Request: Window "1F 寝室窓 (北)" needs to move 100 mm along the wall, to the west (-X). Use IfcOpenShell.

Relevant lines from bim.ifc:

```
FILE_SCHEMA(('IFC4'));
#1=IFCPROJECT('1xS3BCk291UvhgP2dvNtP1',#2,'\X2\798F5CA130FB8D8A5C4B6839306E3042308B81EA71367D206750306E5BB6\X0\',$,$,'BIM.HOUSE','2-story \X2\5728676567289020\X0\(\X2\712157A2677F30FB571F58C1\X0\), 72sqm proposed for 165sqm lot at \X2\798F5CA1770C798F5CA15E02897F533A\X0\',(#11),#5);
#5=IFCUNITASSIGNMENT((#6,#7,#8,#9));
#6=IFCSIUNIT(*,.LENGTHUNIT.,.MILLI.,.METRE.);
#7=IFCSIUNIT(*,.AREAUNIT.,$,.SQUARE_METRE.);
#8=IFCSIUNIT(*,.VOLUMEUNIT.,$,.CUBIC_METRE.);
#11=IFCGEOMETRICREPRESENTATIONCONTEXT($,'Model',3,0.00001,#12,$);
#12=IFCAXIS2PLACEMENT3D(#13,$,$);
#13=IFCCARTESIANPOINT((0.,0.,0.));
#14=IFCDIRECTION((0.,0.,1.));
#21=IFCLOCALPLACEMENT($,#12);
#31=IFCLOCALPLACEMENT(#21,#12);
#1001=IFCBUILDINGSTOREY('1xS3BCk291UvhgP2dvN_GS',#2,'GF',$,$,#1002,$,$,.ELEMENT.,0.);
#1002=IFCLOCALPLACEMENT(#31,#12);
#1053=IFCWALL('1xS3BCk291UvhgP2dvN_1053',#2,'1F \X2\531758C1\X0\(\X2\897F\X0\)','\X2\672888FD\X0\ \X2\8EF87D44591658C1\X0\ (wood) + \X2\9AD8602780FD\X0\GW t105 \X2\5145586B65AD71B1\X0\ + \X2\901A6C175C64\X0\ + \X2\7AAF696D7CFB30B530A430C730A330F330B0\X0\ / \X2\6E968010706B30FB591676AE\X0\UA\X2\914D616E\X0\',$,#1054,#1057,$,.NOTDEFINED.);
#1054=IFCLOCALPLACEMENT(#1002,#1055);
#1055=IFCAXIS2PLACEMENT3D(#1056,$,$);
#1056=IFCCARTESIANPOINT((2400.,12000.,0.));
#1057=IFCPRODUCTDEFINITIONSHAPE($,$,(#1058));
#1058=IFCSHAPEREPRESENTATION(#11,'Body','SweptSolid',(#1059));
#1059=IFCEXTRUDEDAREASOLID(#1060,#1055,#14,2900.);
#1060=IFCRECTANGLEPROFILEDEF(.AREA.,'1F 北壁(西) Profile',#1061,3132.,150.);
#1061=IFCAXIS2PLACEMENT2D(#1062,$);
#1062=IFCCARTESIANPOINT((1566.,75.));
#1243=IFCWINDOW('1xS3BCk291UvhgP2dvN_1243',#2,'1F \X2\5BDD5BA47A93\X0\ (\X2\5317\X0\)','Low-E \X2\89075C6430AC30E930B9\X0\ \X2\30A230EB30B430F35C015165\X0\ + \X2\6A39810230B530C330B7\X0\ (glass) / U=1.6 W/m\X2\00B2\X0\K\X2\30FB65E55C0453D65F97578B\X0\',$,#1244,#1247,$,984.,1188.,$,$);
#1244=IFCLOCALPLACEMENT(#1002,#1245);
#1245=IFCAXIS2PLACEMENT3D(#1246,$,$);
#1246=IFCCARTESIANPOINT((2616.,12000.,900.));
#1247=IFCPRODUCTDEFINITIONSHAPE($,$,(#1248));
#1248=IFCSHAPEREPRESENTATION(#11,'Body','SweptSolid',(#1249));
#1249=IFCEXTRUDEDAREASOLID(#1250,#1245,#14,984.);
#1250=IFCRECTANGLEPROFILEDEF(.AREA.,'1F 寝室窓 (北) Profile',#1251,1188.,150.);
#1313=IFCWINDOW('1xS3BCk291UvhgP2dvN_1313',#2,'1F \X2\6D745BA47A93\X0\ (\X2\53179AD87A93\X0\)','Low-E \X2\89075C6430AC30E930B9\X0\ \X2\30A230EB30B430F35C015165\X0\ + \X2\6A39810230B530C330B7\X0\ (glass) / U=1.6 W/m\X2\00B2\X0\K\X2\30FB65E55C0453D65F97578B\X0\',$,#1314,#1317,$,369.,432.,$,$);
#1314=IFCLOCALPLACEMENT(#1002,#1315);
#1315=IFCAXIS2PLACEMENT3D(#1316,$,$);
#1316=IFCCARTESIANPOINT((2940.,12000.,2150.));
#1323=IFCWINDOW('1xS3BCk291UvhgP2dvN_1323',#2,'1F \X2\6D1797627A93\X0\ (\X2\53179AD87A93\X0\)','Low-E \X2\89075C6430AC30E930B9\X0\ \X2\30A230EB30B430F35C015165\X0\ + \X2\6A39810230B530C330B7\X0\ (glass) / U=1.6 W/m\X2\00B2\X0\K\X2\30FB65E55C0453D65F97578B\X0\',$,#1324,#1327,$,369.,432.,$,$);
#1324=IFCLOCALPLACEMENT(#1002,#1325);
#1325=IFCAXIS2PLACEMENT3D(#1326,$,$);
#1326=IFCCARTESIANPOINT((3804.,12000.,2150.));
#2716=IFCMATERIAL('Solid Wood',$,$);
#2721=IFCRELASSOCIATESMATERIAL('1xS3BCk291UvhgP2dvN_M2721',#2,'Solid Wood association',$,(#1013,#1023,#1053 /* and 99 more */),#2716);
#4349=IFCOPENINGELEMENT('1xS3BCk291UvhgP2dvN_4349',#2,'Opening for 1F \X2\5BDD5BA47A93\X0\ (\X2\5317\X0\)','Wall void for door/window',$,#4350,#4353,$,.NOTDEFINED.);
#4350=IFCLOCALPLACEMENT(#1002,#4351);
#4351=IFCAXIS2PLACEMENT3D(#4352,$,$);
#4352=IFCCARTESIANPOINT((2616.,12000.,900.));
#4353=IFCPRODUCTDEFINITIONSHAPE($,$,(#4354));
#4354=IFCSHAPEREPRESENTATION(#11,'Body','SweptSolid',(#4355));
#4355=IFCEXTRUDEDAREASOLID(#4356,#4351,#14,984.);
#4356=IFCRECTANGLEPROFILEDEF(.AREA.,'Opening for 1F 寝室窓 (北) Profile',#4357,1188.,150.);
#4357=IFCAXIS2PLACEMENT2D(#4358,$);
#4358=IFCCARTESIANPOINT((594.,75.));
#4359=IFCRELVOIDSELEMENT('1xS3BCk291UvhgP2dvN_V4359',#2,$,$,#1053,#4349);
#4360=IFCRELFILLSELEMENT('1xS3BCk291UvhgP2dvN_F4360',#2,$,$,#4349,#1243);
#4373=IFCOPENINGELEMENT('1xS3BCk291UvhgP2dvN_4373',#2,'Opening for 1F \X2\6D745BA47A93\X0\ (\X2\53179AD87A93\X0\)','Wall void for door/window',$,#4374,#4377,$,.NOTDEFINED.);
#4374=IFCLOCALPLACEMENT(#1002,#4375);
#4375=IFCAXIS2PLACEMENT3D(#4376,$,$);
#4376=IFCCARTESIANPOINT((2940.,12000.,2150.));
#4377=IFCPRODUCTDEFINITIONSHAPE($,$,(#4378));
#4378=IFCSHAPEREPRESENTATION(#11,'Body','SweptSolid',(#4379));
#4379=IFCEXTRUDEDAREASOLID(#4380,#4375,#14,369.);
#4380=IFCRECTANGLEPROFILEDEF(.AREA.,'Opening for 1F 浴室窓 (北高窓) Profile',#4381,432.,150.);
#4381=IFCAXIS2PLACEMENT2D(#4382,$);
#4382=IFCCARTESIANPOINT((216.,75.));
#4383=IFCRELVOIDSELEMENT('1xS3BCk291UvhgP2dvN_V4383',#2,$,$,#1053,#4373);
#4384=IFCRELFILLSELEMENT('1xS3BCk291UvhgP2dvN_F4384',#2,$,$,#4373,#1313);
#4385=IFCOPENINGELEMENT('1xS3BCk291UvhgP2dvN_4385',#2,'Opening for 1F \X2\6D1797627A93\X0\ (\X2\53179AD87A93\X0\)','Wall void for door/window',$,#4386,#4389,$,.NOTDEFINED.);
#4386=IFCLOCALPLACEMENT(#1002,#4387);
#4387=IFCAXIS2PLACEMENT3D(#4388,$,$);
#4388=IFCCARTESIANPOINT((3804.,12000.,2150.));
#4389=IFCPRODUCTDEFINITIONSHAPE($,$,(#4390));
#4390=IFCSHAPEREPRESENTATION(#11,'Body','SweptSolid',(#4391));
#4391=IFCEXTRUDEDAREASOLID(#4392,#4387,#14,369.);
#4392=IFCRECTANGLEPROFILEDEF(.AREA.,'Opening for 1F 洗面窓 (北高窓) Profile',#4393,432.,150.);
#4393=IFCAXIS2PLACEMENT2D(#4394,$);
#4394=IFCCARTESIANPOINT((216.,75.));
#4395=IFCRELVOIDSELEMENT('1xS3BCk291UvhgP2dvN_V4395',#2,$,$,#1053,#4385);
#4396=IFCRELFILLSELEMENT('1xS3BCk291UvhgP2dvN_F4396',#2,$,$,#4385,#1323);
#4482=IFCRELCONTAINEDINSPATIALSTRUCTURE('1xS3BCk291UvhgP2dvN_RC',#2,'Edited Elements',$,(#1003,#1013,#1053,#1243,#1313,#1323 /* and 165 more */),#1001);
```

```python
import ifcopenshell
import ifcopenshell.api.geometry
import ifcopenshell.util.placement

model = ifcopenshell.open("bim.ifc")

window = model.by_guid("1xS3BCk291UvhgP2dvN_1243")
opening = window.FillsVoids[0].RelatingOpeningElement
wall = opening.VoidsElements[0].RelatingBuildingElement

wall_matrix = ifcopenshell.util.placement.get_local_placement(wall.ObjectPlacement)
shift = wall_matrix[:3, 0] * -100.0
before = ifcopenshell.util.placement.get_local_placement(window.ObjectPlacement)[:3, 3].copy()

# The window is not placed relative to its opening, so move both.
for product in (opening, window):
    matrix = ifcopenshell.util.placement.get_local_placement(product.ObjectPlacement)
    matrix[:3, 3] += shift
    ifcopenshell.api.geometry.edit_object_placement(model, product=product, matrix=matrix, is_si=False)

after = ifcopenshell.util.placement.get_local_placement(window.ObjectPlacement)[:3, 3]
print("window moved by", (after - before).round(3) + 0.0)

model.write("bim_edited.ifc")
```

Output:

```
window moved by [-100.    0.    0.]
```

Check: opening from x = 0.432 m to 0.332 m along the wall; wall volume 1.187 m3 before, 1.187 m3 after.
